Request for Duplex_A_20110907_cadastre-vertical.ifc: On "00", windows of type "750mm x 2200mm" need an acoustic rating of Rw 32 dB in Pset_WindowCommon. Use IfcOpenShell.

First a look at what the model holds.

```python
import ifcopenshell
import ifcopenshell.util.element

model = ifcopenshell.open("Duplex_A_20110907_cadastre-vertical.ifc")
print(model.schema)
storey = next(s for s in model.by_type("IfcBuildingStorey") if s.Name == "00")
windows = [e for e in ifcopenshell.util.element.get_decomposition(storey) if e.is_a("IfcWindow")]
seen = {}
for e in windows:
    element_type = ifcopenshell.util.element.get_type(e)
    key = (element_type.Name if element_type != e and element_type else None, ifcopenshell.util.element.get_pset(e, "Pset_WindowCommon", "AcousticRating"))
    seen[key] = seen.get(key, 0) + 1
for (name, value), count in sorted(seen.items(), key=str):
    print(count, "x", name, "|", value)
```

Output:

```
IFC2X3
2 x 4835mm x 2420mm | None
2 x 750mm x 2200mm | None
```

```python
import ifcopenshell
import ifcopenshell.api.pset
import ifcopenshell.util.element

model = ifcopenshell.open("Duplex_A_20110907_cadastre-vertical.ifc")

storey = next(s for s in model.by_type("IfcBuildingStorey") if s.Name == "00")
windows = [e for e in ifcopenshell.util.element.get_decomposition(storey) if e.is_a("IfcWindow")]

count = 0
for e in windows:
    element_type = ifcopenshell.util.element.get_type(e)
    if element_type in (None, e) or element_type.Name != "750mm x 2200mm":
        continue
    # add_pset returns the element's existing set when there is one.
    pset = ifcopenshell.api.pset.add_pset(model, product=e, name="Pset_WindowCommon")
    ifcopenshell.api.pset.edit_pset(model, pset=pset, properties={"AcousticRating": "Rw 32 dB"})
    count += 1

print(count, "windows updated")

model.write("Duplex_A_20110907_cadastre-vertical_updated.ifc")
```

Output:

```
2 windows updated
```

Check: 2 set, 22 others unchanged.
